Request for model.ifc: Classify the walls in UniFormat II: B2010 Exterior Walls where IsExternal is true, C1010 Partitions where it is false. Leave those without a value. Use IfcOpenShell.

First a look at what the model holds.

```python
import ifcopenshell
import ifcopenshell.util.element

model = ifcopenshell.open("model.ifc")
print(model.schema)
print("classifications:", [c.Name for c in model.by_type("IfcClassification")])
values = [ifcopenshell.util.element.get_pset(e, "Pset_WallCommon", "IsExternal") for e in model.by_type("IfcWall")]
for value in (True, False, None):
    print("IsExternal", value, values.count(value))
```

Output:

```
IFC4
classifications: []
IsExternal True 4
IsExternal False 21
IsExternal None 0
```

```python
import ifcopenshell
import ifcopenshell.api.classification
import ifcopenshell.util.element

model = ifcopenshell.open("model.ifc")

system = ifcopenshell.api.classification.add_classification(model, classification="UniFormat II")

walls = model.by_type("IfcWall")
external = {e: ifcopenshell.util.element.get_pset(e, "Pset_WallCommon", "IsExternal") for e in walls}
for flag, code, name in ((True, "B2010", "Exterior Walls"), (False, "C1010", "Partitions")):
    products = [e for e in walls if external[e] is flag]
    ifcopenshell.api.classification.add_reference(
        model, products=products, classification=system, identification=code, name=name
    )
    print(code, len(products))

model.write("model-out.ifc")
```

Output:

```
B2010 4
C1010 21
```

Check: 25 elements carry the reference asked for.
